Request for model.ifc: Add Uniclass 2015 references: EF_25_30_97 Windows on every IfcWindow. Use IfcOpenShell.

First a look at what the model holds.

```python
import ifcopenshell

model = ifcopenshell.open("model.ifc")
print(model.schema)
print("classifications:", [c.Name for c in model.by_type("IfcClassification")])
for ifc_class in ("IfcDoor", "IfcRoof", "IfcStair", "IfcWall", "IfcWindow"):
    print(ifc_class, len(model.by_type(ifc_class)))
```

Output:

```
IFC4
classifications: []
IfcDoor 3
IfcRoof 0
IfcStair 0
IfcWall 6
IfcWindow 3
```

```python
import ifcopenshell
import ifcopenshell.api.classification

model = ifcopenshell.open("model.ifc")

system = ifcopenshell.api.classification.add_classification(model, classification="Uniclass 2015")

codes = {
    "IfcWindow": ("EF_25_30_97", "Windows"),
}
for ifc_class, (code, name) in codes.items():
    products = model.by_type(ifc_class)
    ifcopenshell.api.classification.add_reference(
        model, products=products, classification=system, identification=code, name=name
    )
    print(code, len(products))

model.write("model_v2.ifc")
```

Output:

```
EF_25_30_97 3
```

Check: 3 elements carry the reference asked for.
